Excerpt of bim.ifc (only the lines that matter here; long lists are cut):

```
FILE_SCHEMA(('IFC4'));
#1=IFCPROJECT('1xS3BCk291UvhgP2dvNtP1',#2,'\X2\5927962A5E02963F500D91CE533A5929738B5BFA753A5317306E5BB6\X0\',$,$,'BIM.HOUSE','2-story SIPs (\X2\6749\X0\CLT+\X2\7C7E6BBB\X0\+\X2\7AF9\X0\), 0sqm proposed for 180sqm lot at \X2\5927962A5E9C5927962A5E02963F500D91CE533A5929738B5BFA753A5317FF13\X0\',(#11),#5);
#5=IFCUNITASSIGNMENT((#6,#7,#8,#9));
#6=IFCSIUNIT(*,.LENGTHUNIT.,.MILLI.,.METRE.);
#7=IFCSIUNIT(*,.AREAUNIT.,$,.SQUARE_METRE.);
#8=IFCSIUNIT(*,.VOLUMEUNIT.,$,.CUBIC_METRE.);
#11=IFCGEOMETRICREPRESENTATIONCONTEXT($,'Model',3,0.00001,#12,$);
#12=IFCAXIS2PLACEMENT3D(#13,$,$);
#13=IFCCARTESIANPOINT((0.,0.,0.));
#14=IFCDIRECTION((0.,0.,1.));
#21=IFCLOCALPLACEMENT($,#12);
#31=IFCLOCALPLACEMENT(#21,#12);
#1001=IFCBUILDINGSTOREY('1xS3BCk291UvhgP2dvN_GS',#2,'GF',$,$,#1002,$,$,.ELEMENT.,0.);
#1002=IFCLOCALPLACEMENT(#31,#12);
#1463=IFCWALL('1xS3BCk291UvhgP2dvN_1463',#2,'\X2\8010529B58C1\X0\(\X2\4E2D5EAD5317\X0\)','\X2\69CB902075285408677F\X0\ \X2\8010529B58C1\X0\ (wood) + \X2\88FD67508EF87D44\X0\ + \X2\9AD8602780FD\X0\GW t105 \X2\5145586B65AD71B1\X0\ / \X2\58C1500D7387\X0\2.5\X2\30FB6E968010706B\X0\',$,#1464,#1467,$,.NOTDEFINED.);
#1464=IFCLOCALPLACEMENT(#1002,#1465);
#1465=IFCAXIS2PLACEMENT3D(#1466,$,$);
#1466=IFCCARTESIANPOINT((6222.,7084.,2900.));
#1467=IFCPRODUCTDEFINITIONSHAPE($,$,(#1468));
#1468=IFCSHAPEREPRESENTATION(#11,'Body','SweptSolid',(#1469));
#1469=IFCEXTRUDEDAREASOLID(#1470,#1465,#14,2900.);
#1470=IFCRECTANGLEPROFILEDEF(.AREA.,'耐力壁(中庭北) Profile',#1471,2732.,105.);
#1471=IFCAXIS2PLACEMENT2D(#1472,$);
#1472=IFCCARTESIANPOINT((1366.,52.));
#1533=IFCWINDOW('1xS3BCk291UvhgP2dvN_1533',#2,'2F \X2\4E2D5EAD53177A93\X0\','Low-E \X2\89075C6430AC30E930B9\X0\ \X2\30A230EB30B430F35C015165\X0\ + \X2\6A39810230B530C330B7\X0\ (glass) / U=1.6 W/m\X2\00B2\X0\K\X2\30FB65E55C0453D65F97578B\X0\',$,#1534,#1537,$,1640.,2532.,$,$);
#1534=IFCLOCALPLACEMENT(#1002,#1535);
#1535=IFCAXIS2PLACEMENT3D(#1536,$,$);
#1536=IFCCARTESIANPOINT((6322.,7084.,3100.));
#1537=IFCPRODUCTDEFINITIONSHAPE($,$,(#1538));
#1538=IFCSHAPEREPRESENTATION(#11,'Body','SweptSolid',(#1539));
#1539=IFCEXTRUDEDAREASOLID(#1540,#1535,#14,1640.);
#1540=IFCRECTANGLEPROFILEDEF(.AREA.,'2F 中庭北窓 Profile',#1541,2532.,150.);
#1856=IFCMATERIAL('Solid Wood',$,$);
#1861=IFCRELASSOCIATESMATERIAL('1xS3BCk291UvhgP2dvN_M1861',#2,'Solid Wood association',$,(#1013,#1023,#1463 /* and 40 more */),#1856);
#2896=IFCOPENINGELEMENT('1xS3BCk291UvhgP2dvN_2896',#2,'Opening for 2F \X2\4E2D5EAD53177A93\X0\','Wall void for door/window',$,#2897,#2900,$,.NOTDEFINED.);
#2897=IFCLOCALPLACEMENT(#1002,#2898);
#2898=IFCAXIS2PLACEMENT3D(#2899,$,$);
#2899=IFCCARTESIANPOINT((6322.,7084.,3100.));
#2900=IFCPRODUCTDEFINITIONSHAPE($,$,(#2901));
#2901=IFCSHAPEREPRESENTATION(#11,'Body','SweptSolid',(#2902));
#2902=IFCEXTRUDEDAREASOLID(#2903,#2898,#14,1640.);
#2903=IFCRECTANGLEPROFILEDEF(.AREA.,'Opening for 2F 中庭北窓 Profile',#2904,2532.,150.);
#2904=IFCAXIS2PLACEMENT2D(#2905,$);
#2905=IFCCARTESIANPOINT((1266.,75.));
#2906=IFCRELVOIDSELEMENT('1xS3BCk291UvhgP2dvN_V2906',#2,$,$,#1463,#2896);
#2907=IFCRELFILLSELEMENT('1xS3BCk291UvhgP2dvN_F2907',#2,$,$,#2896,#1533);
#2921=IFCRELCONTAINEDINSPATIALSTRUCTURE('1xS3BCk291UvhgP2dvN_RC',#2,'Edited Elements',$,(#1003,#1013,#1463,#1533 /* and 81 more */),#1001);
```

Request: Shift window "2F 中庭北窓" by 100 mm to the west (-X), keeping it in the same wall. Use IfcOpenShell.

```python
import ifcopenshell
import ifcopenshell.api.geometry
import ifcopenshell.util.placement
import ifcopenshell.util.unit

model = ifcopenshell.open("bim.ifc")
unit_scale = ifcopenshell.util.unit.calculate_unit_scale(model)

window = model.by_id(1533)
opening = window.FillsVoids[0].RelatingOpeningElement
wall = opening.VoidsElements[0].RelatingBuildingElement

wall_matrix = ifcopenshell.util.placement.get_local_placement(wall.ObjectPlacement)
shift = wall_matrix[:3, 0] * -0.1 / unit_scale
before = ifcopenshell.util.placement.get_local_placement(window.ObjectPlacement)[:3, 3].copy()

# The window is not placed relative to its opening, so move both.
for product in (opening, window):
    matrix = ifcopenshell.util.placement.get_local_placement(product.ObjectPlacement)
    matrix[:3, 3] += shift
    ifcopenshell.api.geometry.edit_object_placement(model, product=product, matrix=matrix, is_si=False)

after = ifcopenshell.util.placement.get_local_placement(window.ObjectPlacement)[:3, 3]
print("window moved by", (after - before).round(3) + 0.0)

model.write("bim-out.ifc")
```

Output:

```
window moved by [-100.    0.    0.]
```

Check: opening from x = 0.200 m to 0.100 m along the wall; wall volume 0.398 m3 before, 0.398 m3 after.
